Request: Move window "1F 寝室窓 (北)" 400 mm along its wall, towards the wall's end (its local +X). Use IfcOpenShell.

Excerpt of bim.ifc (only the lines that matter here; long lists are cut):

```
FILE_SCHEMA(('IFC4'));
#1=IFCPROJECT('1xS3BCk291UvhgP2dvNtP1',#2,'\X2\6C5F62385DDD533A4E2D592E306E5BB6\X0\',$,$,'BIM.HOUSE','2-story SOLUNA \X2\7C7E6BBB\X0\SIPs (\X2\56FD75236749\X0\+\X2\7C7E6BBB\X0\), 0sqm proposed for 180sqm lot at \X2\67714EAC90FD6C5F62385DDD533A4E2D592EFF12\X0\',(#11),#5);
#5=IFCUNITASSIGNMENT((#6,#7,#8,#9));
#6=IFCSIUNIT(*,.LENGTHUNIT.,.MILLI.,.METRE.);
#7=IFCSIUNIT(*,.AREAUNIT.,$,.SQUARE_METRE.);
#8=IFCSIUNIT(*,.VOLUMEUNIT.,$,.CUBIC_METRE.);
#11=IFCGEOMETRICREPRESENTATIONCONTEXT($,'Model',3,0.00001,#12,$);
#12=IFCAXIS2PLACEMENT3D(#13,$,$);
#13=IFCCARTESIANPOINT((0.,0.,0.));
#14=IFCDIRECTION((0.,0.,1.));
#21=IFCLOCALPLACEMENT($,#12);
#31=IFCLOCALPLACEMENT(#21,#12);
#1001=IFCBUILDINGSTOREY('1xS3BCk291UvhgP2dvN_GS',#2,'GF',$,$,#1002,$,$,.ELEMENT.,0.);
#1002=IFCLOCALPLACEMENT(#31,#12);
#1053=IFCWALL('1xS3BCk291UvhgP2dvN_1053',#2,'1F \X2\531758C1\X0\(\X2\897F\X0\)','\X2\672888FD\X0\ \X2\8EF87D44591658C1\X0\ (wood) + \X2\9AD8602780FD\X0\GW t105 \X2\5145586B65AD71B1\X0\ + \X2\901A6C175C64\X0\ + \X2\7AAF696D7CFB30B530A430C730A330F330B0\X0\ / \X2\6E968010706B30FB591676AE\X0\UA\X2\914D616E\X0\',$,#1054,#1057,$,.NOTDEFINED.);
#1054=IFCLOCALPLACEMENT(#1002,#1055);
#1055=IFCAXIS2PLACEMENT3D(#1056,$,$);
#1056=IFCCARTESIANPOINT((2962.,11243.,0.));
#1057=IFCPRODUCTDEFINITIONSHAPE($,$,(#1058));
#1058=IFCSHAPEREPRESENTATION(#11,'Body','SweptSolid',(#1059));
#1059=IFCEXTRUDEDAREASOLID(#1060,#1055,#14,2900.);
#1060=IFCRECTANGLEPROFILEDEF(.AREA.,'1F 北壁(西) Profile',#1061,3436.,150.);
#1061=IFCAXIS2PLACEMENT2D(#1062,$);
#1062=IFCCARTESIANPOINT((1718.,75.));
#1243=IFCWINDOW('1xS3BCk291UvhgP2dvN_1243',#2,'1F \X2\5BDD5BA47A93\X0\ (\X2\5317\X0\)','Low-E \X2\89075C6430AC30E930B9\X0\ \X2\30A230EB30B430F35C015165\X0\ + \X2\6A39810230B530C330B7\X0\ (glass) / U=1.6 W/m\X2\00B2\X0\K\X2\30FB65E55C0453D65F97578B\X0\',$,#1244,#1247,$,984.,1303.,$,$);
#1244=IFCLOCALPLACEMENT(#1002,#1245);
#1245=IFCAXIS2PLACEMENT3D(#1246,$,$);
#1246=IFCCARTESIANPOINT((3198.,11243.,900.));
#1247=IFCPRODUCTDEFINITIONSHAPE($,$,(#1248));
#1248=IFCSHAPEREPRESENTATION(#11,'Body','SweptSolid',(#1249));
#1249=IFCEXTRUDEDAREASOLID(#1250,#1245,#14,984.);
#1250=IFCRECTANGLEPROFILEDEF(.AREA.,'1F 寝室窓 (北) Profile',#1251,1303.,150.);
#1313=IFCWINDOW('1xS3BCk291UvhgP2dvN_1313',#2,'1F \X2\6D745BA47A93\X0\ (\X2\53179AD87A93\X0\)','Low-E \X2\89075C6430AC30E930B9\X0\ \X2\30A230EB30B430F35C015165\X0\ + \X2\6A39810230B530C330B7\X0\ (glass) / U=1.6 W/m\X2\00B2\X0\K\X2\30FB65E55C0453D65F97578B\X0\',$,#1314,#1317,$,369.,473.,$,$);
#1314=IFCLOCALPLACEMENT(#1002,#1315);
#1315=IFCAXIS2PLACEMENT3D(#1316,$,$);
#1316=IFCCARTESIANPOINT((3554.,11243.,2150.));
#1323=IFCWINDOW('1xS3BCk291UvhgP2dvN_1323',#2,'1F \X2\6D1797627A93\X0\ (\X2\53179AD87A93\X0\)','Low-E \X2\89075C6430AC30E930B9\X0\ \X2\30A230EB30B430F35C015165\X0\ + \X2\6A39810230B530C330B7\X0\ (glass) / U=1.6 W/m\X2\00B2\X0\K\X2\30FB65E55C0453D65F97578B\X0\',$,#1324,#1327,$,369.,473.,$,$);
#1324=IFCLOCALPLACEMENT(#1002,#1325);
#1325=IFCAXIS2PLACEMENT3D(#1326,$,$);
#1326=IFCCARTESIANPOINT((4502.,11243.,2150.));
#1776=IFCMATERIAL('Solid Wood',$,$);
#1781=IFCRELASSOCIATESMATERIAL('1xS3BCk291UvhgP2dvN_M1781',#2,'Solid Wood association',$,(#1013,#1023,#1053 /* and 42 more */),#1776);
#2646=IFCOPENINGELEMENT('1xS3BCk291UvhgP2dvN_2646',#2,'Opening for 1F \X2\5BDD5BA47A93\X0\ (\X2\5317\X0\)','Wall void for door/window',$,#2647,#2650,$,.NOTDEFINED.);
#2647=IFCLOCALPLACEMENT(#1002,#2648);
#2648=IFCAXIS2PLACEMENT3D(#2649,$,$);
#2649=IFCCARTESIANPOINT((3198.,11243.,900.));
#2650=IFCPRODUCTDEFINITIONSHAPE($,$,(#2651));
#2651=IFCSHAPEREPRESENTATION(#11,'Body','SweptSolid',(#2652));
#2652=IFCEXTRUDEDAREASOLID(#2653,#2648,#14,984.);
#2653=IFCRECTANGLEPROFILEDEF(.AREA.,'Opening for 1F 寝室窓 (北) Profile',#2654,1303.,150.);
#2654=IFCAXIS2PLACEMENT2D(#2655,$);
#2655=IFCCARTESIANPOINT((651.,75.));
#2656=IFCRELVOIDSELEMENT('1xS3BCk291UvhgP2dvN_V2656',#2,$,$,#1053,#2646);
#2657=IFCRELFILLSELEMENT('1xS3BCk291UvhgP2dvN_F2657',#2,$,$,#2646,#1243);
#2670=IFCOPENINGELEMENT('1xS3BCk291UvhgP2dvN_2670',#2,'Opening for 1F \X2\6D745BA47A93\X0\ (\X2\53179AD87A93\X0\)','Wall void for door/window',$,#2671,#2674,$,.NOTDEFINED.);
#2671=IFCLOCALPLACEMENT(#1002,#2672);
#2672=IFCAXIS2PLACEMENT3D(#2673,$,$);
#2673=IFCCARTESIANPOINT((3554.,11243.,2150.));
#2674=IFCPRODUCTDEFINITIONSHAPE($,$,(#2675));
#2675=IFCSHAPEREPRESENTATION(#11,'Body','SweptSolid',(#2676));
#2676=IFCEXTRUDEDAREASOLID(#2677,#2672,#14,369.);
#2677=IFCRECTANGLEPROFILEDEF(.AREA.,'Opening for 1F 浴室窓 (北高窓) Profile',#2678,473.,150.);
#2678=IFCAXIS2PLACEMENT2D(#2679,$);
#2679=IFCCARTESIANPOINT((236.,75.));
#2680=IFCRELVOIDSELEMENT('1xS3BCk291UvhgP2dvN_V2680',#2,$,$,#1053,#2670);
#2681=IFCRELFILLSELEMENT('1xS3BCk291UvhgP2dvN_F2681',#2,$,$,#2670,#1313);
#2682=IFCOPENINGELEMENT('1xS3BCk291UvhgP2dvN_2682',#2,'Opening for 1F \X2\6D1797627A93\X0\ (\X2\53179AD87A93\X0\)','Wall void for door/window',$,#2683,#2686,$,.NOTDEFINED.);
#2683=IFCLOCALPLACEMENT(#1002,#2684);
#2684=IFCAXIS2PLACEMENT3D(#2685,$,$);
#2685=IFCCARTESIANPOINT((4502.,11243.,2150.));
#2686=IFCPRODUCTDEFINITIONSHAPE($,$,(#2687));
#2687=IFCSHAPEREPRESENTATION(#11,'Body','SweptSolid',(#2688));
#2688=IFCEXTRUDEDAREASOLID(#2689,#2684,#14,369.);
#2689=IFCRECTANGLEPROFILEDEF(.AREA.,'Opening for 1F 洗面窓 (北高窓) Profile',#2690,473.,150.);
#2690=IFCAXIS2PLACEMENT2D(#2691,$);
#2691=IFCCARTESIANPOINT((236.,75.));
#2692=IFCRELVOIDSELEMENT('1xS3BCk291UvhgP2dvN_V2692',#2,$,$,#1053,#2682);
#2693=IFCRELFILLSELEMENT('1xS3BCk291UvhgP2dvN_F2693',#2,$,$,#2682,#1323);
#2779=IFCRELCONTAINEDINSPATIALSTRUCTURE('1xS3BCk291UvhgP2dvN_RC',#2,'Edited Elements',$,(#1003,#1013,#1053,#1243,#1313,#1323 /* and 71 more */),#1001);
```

```python
import ifcopenshell
import ifcopenshell.api.geometry
import ifcopenshell.util.placement

model = ifcopenshell.open("bim.ifc")

window = model.by_guid("1xS3BCk291UvhgP2dvN_1243")
opening = window.FillsVoids[0].RelatingOpeningElement
wall = opening.VoidsElements[0].RelatingBuildingElement

wall_matrix = ifcopenshell.util.placement.get_local_placement(wall.ObjectPlacement)
shift = wall_matrix[:3, 0] * 400.0
before = ifcopenshell.util.placement.get_local_placement(window.ObjectPlacement)[:3, 3].copy()

# The window is not placed relative to its opening, so move both.
for product in (opening, window):
    matrix = ifcopenshell.util.placement.get_local_placement(product.ObjectPlacement)
    matrix[:3, 3] += shift
    ifcopenshell.api.geometry.edit_object_placement(model, product=product, matrix=matrix, is_si=False)

after = ifcopenshell.util.placement.get_local_placement(window.ObjectPlacement)[:3, 3]
print("window moved by", (after - before).round(3) + 0.0)

model.write("bim_rev.ifc")
```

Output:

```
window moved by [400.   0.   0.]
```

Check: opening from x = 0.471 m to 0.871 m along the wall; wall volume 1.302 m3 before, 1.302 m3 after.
